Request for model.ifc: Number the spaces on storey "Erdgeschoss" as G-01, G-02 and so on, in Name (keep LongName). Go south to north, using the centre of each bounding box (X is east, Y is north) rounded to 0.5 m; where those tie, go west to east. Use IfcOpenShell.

First a look at what the model holds.

```python
import ifcopenshell
import ifcopenshell.util.element
import ifcopenshell.util.placement

model = ifcopenshell.open("model.ifc")
print(model.schema)
storey = next(s for s in model.by_type("IfcBuildingStorey") if s.Name == "Erdgeschoss")
spaces = [e for e in ifcopenshell.util.element.get_decomposition(storey) if e.is_a("IfcSpace")]
for e in sorted(spaces, key=lambda e: e.id()):
    origin = ifcopenshell.util.placement.get_local_placement(e.ObjectPlacement)[:3, 3]
    print(e.id(), e.Name, e.LongName, origin.round(2) + 0.0, sep=" | ")
```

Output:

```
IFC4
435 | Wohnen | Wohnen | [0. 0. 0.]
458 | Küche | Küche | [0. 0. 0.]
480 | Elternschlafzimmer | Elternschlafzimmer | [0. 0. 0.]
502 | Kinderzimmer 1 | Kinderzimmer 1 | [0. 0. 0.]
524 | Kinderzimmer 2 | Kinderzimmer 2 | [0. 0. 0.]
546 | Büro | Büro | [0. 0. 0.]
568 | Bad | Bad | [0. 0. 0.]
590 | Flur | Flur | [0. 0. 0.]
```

```python
import ifcopenshell
import ifcopenshell.geom
import ifcopenshell.util.element
import ifcopenshell.util.shape

model = ifcopenshell.open("model.ifc")
settings = ifcopenshell.geom.settings()
settings.set("use-world-coords", True)


def centre(element):
    shape = ifcopenshell.geom.create_shape(settings, element)
    return ifcopenshell.util.shape.get_bbox_centroid(shape.geometry)


storey = next(s for s in model.by_type("IfcBuildingStorey") if s.Name == "Erdgeschoss")
spaces = [e for e in ifcopenshell.util.element.get_decomposition(storey) if e.is_a("IfcSpace")]

# Insertion points can sit at a corner or the storey origin, so sort by the geometry (in metres).
centres = {e: centre(e) for e in spaces}
spaces.sort(key=lambda e: (round(centres[e][1] / 0.5), centres[e][0]))

for i, e in enumerate(spaces, start=1):
    number = f"G-{i:02d}"
    e.Name = number
    print(e.id(), number)

model.write("model-out.ifc")
```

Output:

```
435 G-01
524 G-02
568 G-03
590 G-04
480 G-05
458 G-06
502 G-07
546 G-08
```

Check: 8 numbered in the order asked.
